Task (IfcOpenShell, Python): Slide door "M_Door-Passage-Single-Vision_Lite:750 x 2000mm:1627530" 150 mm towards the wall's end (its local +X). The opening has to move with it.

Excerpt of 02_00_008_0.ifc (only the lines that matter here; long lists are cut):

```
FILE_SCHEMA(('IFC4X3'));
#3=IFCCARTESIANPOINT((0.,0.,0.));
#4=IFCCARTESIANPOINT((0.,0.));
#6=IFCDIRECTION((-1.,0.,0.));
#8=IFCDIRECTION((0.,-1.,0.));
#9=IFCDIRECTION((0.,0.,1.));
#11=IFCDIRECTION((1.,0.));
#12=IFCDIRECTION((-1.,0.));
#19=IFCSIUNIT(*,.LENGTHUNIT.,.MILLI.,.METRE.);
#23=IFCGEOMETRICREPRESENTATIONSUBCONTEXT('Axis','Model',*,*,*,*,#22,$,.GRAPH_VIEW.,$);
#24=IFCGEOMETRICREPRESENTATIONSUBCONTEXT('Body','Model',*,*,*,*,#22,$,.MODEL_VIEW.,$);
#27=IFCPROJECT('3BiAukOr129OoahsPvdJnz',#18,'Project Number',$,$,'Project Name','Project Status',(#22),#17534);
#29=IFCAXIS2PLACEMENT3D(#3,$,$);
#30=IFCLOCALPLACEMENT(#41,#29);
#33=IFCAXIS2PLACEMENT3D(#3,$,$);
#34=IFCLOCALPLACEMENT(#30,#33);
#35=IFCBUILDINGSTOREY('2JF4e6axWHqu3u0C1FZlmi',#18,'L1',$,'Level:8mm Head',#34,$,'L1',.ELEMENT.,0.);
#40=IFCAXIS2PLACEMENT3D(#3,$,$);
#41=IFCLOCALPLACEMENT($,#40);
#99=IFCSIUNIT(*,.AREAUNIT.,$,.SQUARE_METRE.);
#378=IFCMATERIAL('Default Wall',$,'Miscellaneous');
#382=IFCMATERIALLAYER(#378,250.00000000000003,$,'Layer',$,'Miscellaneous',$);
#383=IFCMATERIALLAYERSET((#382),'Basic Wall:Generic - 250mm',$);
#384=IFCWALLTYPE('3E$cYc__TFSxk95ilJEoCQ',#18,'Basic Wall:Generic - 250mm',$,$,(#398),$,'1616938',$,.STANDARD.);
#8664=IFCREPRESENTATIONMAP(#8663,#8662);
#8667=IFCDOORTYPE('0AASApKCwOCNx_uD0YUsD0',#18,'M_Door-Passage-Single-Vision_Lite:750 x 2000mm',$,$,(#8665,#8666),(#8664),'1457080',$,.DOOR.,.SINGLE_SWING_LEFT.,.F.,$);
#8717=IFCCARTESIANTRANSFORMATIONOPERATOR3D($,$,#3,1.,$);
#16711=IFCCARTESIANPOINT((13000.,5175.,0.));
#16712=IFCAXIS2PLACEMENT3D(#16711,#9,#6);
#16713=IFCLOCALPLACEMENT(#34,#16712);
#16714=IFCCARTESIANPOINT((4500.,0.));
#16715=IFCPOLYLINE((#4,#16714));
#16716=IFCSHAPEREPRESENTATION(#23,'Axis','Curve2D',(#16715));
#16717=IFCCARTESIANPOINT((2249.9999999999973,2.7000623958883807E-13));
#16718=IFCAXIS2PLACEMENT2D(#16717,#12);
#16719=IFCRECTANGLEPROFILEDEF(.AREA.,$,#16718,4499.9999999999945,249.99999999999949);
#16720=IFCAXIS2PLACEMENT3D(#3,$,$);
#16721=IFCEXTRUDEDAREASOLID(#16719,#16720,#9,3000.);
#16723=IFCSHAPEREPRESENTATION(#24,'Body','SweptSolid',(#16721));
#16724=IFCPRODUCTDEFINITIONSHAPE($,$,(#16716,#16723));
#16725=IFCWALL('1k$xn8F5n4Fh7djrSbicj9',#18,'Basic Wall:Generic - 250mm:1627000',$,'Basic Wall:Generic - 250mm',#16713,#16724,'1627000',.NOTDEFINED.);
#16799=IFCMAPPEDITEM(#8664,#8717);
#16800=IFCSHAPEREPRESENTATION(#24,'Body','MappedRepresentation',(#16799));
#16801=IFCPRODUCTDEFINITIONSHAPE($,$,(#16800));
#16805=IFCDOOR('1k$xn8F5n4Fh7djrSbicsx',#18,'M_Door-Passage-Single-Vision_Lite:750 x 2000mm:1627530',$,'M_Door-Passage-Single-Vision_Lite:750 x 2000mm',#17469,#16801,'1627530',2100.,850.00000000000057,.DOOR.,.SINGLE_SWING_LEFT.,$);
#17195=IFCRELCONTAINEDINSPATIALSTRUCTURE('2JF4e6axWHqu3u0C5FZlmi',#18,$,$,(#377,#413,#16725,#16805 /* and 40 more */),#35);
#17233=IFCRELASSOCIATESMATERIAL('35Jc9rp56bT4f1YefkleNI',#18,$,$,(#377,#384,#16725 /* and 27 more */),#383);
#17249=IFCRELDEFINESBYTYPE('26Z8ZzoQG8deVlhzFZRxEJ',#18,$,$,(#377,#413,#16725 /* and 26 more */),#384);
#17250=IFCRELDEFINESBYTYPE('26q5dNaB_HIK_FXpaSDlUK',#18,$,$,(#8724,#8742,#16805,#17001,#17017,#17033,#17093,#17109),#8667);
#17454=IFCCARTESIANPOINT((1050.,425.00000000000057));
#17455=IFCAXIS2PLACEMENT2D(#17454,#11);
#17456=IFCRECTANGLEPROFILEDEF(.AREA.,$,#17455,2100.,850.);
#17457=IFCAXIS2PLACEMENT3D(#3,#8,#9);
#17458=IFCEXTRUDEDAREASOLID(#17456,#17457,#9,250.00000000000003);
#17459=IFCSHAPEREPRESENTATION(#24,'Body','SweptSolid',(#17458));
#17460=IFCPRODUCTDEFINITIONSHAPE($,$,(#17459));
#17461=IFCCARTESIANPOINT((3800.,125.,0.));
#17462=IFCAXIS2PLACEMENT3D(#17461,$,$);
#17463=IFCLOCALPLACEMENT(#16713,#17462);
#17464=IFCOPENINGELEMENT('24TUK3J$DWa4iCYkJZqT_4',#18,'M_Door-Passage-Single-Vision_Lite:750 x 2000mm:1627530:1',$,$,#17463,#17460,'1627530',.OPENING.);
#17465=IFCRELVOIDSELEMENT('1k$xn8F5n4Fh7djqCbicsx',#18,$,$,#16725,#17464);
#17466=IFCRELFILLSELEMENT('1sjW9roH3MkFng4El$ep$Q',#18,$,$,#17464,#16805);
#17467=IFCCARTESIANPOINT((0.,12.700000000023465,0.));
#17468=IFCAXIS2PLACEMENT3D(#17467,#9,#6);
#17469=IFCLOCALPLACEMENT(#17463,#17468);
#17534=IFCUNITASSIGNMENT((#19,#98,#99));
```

```python
import ifcopenshell
import ifcopenshell.api.geometry
import ifcopenshell.util.placement
import ifcopenshell.util.unit

model = ifcopenshell.open("02_00_008_0.ifc")
unit_scale = ifcopenshell.util.unit.calculate_unit_scale(model)

door = model.by_guid("1k$xn8F5n4Fh7djrSbicsx")
opening = door.FillsVoids[0].RelatingOpeningElement
wall = opening.VoidsElements[0].RelatingBuildingElement

wall_matrix = ifcopenshell.util.placement.get_local_placement(wall.ObjectPlacement)
shift = wall_matrix[:3, 0] * 0.15 / unit_scale
before = ifcopenshell.util.placement.get_local_placement(door.ObjectPlacement)[:3, 3].copy()

# The door is placed relative to its opening, so it follows when the opening moves.
matrix = ifcopenshell.util.placement.get_local_placement(opening.ObjectPlacement)
matrix[:3, 3] += shift
ifcopenshell.api.geometry.edit_object_placement(
    model, product=opening, matrix=matrix, is_si=False, should_transform_children=True
)

after = ifcopenshell.util.placement.get_local_placement(door.ObjectPlacement)[:3, 3]
print("door moved by", (after - before).round(3) + 0.0)

model.write("02_00_008_0_updated.ifc")
```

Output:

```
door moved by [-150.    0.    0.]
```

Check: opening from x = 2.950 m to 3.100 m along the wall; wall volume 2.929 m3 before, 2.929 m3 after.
